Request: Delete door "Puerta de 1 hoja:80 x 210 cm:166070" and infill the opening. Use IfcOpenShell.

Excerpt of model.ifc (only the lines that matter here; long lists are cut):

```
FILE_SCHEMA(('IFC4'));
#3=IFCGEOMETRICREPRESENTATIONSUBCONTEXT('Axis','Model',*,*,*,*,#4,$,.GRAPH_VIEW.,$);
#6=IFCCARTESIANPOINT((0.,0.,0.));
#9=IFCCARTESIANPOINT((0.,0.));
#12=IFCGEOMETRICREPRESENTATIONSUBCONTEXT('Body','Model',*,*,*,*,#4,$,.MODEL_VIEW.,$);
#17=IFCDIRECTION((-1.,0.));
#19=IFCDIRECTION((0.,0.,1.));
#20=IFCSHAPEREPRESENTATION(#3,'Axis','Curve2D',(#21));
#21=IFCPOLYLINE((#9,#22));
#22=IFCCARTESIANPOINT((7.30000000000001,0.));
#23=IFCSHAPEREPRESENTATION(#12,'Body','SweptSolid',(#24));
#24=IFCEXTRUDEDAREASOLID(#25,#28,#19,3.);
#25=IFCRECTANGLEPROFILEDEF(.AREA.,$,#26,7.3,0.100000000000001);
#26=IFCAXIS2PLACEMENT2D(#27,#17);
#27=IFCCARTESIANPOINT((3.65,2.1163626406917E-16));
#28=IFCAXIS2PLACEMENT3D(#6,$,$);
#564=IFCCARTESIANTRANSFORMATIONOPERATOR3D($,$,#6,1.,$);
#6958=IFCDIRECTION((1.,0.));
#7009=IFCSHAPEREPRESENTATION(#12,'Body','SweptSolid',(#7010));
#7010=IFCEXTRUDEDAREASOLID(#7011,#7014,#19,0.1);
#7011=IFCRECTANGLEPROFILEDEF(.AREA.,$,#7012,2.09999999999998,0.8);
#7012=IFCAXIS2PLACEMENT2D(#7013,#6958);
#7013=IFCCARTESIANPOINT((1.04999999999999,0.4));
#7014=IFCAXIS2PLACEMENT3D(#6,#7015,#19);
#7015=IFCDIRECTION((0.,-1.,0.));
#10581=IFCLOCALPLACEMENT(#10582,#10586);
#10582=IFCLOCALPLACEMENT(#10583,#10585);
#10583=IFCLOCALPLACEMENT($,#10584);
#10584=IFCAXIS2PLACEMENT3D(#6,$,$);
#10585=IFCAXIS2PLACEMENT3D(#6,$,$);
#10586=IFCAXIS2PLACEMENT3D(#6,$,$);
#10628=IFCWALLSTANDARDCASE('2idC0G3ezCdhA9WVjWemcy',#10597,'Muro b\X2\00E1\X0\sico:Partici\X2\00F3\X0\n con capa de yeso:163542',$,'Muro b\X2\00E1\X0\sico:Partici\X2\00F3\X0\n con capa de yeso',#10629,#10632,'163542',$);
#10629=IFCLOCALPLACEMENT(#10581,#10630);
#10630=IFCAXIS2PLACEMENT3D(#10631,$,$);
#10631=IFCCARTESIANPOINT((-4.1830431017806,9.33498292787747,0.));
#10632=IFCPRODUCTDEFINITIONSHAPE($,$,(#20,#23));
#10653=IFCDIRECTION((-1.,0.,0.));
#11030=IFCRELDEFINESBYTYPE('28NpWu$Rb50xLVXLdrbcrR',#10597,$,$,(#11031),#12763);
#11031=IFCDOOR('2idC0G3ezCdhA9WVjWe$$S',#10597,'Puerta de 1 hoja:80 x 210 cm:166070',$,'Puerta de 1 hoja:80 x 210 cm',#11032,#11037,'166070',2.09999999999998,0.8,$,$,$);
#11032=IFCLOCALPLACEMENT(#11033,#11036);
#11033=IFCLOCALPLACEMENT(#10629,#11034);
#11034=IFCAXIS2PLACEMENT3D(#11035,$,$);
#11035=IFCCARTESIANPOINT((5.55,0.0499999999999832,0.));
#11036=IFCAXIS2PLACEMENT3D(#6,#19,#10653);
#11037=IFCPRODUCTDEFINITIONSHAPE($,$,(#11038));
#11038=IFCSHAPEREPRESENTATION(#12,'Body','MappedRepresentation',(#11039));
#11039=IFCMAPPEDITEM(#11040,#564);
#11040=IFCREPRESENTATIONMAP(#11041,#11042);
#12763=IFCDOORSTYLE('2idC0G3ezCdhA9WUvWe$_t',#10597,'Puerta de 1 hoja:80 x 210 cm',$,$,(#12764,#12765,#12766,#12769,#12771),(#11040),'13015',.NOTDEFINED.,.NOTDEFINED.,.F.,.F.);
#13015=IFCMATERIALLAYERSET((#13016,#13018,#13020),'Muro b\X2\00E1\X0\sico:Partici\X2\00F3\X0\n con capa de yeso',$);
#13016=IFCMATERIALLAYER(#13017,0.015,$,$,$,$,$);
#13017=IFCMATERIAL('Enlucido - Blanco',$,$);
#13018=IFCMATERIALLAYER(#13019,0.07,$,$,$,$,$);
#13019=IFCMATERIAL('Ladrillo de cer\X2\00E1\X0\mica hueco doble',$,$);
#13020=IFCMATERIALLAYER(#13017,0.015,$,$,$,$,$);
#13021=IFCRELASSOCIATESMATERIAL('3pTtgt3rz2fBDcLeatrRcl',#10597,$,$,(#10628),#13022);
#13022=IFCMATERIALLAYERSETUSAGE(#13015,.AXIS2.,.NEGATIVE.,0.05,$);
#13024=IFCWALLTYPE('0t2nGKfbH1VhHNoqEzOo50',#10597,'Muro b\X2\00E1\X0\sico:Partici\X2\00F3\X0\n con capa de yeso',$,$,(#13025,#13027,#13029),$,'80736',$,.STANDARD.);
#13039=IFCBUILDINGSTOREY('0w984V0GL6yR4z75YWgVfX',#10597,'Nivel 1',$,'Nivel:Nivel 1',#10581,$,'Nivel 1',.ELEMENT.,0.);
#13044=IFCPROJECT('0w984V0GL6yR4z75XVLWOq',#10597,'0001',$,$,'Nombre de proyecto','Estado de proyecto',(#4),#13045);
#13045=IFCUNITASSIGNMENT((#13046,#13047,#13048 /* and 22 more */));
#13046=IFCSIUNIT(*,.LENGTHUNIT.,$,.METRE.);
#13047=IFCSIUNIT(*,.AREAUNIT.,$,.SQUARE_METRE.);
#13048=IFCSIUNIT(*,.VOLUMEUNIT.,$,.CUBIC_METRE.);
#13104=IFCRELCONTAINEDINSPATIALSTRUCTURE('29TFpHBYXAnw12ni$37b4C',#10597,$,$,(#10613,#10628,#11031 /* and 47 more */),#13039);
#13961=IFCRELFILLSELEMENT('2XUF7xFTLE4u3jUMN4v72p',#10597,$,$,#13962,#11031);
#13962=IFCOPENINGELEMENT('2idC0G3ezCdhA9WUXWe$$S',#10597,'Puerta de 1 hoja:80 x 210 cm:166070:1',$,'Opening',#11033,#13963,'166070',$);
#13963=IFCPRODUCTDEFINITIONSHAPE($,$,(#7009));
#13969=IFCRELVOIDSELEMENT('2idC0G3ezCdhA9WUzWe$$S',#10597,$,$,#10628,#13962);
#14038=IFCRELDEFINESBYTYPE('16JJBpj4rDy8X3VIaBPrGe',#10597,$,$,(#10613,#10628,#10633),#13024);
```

```python
import ifcopenshell
import ifcopenshell.api.feature
import ifcopenshell.api.root
import ifcopenshell.geom
import ifcopenshell.util.shape

model = ifcopenshell.open("model.ifc")
settings = ifcopenshell.geom.settings()


def volume(element):
    """Net volume in cubic metres, openings subtracted."""
    shape = ifcopenshell.geom.create_shape(settings, element)
    return ifcopenshell.util.shape.get_volume(shape.geometry)


door = model.by_guid("2idC0G3ezCdhA9WVjWe$$S")
opening = door.FillsVoids[0].RelatingOpeningElement
wall = opening.VoidsElements[0].RelatingBuildingElement
before = volume(wall)

ifcopenshell.api.root.remove_product(model, product=door)
ifcopenshell.api.feature.remove_feature(model, feature=opening)

after = volume(wall)

print(f"wall volume {before:.3f} -> {after:.3f} m3")

model.write("model_v2.ifc")
```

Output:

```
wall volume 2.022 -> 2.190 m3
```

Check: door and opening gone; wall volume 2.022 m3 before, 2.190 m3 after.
